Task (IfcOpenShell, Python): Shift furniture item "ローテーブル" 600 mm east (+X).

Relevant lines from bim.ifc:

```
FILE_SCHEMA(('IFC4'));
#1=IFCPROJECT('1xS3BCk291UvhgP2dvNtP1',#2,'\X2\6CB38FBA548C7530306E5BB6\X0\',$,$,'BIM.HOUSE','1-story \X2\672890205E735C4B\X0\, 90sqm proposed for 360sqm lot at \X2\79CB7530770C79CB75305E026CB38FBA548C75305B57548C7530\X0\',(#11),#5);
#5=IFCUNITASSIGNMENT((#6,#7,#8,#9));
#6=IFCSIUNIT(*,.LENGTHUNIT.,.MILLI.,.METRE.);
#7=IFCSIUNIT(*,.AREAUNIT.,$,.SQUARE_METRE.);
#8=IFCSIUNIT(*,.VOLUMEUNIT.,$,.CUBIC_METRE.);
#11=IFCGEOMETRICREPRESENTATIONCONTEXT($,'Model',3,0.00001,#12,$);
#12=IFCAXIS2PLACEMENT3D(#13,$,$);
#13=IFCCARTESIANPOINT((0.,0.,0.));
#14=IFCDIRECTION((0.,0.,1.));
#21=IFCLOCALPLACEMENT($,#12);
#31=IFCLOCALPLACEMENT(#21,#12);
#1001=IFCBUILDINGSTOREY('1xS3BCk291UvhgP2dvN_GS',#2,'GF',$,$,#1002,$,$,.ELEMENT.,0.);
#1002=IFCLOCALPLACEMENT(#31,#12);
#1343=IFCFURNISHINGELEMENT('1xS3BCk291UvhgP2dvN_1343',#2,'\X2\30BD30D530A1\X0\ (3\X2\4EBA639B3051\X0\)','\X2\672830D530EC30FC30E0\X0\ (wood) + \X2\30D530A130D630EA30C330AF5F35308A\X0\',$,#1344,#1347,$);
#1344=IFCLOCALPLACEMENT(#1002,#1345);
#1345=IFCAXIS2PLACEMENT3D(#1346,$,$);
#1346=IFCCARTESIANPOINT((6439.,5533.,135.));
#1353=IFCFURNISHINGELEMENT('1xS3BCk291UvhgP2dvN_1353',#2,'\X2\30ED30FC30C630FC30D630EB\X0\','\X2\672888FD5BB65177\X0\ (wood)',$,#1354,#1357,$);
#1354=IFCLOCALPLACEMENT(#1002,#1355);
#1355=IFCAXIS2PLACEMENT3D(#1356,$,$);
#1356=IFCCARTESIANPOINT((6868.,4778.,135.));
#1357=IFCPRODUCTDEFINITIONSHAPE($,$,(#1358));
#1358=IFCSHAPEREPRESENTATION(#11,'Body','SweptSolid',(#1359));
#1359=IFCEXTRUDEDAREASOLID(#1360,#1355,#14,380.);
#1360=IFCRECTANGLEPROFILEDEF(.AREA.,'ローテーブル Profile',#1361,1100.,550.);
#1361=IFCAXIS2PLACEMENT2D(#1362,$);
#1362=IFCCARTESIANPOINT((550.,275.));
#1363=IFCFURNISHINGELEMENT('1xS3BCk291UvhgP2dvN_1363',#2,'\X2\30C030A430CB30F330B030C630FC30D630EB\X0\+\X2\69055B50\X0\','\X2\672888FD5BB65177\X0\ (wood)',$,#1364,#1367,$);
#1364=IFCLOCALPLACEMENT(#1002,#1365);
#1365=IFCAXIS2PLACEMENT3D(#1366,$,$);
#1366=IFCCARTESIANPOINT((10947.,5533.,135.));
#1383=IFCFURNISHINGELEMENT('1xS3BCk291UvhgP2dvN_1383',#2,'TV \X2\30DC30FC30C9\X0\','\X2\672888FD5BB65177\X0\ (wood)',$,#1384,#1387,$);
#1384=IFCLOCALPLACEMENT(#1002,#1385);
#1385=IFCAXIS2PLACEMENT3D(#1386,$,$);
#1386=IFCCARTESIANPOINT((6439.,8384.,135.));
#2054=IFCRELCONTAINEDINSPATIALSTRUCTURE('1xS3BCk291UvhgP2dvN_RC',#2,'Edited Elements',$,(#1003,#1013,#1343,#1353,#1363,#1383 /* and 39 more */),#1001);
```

```python
import ifcopenshell
import ifcopenshell.api.geometry
import ifcopenshell.util.placement
import ifcopenshell.util.unit

model = ifcopenshell.open("bim.ifc")
unit_scale = ifcopenshell.util.unit.calculate_unit_scale(model)

item = model.by_id(1353)
matrix = ifcopenshell.util.placement.get_local_placement(item.ObjectPlacement)
matrix[0, 3] += 0.6 / unit_scale
ifcopenshell.api.geometry.edit_object_placement(model, product=item, matrix=matrix, is_si=False)

print(ifcopenshell.util.placement.get_local_placement(item.ObjectPlacement).round(3) + 0.0)

model.write("bim_updated.ifc")
```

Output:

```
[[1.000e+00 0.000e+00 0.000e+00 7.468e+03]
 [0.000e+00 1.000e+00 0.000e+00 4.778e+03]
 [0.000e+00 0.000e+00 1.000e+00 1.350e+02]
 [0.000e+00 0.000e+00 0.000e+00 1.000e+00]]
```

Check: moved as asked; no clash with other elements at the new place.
